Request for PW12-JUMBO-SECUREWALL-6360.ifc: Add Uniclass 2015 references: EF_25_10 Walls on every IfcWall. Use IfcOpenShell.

First a look at what the model holds.

```python
import ifcopenshell

model = ifcopenshell.open("PW12-JUMBO-SECUREWALL-6360.ifc")
print(model.schema)
print("classifications:", [c.Name for c in model.by_type("IfcClassification")])
for ifc_class in ("IfcDoor", "IfcRoof", "IfcStair", "IfcWall", "IfcWindow"):
    print(ifc_class, len(model.by_type(ifc_class)))
```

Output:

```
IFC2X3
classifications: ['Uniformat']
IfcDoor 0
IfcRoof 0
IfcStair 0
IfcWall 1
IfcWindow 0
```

```python
import ifcopenshell
import ifcopenshell.api.classification

model = ifcopenshell.open("PW12-JUMBO-SECUREWALL-6360.ifc")

# IFC2X3 requires Source and Edition and has no link from the project to the system.
system = model.create_entity("IfcClassification", Source="NBS", Edition="2015", Name="Uniclass 2015")

codes = {
    "IfcWall": ("EF_25_10", "Walls"),
}
for ifc_class, (code, name) in codes.items():
    products = model.by_type(ifc_class)
    ifcopenshell.api.classification.add_reference(
        model, products=products, classification=system, identification=code, name=name
    )
    print(code, len(products))

model.write("PW12-JUMBO-SECUREWALL-6360-out.ifc")
```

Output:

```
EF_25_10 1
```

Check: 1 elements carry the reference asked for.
